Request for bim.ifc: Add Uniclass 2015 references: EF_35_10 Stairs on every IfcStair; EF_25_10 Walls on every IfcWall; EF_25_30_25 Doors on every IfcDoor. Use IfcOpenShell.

First a look at what the model holds.

```python
import ifcopenshell

model = ifcopenshell.open("bim.ifc")
print(model.schema)
print("classifications:", [c.Name for c in model.by_type("IfcClassification")])
for ifc_class in ("IfcDoor", "IfcRoof", "IfcStair", "IfcWall", "IfcWindow"):
    print(ifc_class, len(model.by_type(ifc_class)))
```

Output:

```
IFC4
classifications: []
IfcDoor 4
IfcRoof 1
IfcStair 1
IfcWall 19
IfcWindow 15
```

```python
import ifcopenshell
import ifcopenshell.api.classification

model = ifcopenshell.open("bim.ifc")

system = ifcopenshell.api.classification.add_classification(model, classification="Uniclass 2015")

codes = {
    "IfcStair": ("EF_35_10", "Stairs"),
    "IfcWall": ("EF_25_10", "Walls"),
    "IfcDoor": ("EF_25_30_25", "Doors"),
}
for ifc_class, (code, name) in codes.items():
    products = model.by_type(ifc_class)
    ifcopenshell.api.classification.add_reference(
        model, products=products, classification=system, identification=code, name=name
    )
    print(code, len(products))

model.write("bim_v2.ifc")
```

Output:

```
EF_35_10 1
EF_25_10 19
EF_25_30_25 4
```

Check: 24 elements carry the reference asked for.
